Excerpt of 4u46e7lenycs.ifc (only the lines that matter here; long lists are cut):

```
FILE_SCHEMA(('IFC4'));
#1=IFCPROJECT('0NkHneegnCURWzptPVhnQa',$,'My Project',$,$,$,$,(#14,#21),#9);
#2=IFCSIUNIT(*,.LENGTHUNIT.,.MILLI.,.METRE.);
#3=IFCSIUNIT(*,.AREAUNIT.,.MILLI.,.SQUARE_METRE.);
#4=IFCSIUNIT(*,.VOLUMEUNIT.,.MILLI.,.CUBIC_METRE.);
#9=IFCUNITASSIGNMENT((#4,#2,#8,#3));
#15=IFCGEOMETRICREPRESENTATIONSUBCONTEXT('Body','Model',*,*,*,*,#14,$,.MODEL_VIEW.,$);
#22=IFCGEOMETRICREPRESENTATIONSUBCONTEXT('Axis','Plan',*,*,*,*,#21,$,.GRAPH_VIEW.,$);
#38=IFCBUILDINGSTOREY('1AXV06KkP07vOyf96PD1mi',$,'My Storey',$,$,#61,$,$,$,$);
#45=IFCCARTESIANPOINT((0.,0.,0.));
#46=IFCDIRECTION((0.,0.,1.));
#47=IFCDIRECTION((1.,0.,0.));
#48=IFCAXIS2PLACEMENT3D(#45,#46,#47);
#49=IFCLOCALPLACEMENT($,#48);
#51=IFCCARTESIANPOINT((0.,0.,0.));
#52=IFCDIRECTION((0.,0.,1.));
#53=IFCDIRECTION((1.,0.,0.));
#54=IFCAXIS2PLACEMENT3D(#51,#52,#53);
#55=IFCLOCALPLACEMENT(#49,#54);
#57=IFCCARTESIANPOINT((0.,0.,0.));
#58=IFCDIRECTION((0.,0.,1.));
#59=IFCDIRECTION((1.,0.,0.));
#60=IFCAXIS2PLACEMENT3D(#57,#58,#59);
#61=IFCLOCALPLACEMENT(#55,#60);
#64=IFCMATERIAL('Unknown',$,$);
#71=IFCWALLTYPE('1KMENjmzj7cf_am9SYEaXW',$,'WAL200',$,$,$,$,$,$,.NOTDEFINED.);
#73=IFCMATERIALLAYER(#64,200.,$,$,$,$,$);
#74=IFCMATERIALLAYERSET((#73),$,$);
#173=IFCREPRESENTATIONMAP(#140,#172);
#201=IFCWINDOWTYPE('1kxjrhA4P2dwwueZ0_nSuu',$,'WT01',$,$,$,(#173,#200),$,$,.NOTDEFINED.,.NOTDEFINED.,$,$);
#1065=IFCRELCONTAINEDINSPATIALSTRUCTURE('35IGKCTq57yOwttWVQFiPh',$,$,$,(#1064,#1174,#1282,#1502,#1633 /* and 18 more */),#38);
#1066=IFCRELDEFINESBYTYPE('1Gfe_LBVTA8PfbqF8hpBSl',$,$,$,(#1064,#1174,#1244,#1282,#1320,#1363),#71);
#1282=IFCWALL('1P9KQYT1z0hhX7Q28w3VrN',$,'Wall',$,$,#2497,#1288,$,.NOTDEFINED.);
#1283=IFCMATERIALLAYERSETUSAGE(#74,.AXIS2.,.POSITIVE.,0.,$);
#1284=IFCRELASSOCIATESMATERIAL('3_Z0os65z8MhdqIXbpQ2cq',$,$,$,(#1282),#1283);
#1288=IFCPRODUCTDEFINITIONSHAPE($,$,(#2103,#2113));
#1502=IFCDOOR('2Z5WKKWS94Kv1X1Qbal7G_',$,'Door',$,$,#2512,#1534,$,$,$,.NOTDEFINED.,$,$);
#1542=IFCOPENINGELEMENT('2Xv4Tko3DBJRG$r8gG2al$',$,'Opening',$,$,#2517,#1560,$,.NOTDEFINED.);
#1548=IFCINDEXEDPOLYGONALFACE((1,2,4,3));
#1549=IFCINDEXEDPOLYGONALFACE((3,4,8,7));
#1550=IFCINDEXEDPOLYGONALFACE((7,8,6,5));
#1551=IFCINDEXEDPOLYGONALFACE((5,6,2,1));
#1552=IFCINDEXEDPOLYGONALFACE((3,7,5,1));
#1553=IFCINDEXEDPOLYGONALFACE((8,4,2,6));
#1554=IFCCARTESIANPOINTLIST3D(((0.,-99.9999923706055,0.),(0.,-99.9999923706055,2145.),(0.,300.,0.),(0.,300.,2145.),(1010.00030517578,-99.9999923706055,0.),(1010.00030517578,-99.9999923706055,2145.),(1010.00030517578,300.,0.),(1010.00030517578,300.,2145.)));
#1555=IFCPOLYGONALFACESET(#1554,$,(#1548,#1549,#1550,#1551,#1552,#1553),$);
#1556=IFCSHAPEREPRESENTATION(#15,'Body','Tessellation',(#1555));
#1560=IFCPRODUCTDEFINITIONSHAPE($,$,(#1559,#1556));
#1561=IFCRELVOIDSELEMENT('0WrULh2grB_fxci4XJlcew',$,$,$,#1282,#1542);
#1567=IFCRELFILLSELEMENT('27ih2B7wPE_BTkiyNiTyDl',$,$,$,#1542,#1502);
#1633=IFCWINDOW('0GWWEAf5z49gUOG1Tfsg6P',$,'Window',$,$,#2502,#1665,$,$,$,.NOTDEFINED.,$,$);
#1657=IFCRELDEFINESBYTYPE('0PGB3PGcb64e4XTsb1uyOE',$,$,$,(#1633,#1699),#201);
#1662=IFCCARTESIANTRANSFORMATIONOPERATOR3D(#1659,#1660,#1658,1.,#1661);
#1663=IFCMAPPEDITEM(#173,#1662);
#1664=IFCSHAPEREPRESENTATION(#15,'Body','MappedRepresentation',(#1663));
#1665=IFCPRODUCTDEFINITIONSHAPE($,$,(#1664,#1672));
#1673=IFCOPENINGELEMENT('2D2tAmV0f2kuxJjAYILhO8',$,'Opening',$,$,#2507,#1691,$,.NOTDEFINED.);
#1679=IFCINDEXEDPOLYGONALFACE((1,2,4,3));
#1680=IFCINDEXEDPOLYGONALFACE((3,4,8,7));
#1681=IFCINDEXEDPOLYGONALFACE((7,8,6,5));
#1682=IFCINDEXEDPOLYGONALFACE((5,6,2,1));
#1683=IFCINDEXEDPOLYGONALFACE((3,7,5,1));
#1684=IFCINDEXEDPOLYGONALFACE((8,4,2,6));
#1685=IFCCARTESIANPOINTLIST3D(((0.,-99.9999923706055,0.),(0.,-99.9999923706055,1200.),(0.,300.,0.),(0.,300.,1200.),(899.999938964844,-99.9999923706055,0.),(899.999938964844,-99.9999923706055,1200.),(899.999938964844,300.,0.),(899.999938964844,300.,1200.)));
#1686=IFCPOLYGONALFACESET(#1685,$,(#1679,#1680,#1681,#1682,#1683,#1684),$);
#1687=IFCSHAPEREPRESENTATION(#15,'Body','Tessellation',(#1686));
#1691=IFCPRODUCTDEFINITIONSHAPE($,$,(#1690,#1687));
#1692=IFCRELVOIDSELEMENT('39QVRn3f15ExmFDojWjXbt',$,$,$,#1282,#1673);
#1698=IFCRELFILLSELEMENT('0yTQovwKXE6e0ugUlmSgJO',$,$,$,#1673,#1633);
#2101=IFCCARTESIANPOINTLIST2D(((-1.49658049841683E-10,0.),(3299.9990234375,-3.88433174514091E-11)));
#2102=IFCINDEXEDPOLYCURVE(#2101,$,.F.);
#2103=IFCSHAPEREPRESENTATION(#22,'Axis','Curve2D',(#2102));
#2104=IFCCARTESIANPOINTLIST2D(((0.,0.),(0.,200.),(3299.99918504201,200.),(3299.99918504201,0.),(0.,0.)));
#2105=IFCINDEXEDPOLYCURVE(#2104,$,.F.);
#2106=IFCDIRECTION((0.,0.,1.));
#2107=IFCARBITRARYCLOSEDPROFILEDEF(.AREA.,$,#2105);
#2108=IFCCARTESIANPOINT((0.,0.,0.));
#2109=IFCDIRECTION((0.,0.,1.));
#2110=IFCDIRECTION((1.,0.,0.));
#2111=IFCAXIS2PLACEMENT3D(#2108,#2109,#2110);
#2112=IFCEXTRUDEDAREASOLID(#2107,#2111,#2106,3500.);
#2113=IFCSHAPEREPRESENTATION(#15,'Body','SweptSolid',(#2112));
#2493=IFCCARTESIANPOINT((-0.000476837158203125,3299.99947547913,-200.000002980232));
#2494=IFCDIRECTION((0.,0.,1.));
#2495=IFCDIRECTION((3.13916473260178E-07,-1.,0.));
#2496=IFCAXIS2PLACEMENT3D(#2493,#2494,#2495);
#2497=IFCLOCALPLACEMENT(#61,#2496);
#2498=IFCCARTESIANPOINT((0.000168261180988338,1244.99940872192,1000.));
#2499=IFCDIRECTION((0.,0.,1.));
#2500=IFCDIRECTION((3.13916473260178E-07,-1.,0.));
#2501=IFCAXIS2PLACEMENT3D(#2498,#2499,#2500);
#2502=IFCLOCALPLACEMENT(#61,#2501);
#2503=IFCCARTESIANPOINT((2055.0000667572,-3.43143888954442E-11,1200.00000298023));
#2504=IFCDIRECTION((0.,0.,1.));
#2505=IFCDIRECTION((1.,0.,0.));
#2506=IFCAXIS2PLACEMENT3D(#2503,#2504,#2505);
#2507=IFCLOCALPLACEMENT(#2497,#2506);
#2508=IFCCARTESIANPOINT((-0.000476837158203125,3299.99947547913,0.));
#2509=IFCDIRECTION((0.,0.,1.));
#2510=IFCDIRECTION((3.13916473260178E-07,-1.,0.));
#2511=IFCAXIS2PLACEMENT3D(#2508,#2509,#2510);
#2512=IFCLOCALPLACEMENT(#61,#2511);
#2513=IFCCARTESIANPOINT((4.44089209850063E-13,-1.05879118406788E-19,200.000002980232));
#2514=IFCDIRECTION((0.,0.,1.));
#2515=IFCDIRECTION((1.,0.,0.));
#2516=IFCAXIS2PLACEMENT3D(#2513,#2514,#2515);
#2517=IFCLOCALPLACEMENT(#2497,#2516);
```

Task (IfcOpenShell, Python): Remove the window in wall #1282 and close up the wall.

```python
import ifcopenshell
import ifcopenshell.api.feature
import ifcopenshell.api.root
import ifcopenshell.geom
import ifcopenshell.util.shape

model = ifcopenshell.open("4u46e7lenycs.ifc")
settings = ifcopenshell.geom.settings()


def volume(element):
    """Net volume in cubic metres, openings subtracted."""
    shape = ifcopenshell.geom.create_shape(settings, element)
    return ifcopenshell.util.shape.get_volume(shape.geometry)


window = model.by_guid("0GWWEAf5z49gUOG1Tfsg6P")
opening = window.FillsVoids[0].RelatingOpeningElement
wall = opening.VoidsElements[0].RelatingBuildingElement
before = volume(wall)

ifcopenshell.api.root.remove_product(model, product=window)
ifcopenshell.api.feature.remove_feature(model, feature=opening)

after = volume(wall)

print(f"wall volume {before:.3f} -> {after:.3f} m3")

model.write("4u46e7lenycs_updated.ifc")
```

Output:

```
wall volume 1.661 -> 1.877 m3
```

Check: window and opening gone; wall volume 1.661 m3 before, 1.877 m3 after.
